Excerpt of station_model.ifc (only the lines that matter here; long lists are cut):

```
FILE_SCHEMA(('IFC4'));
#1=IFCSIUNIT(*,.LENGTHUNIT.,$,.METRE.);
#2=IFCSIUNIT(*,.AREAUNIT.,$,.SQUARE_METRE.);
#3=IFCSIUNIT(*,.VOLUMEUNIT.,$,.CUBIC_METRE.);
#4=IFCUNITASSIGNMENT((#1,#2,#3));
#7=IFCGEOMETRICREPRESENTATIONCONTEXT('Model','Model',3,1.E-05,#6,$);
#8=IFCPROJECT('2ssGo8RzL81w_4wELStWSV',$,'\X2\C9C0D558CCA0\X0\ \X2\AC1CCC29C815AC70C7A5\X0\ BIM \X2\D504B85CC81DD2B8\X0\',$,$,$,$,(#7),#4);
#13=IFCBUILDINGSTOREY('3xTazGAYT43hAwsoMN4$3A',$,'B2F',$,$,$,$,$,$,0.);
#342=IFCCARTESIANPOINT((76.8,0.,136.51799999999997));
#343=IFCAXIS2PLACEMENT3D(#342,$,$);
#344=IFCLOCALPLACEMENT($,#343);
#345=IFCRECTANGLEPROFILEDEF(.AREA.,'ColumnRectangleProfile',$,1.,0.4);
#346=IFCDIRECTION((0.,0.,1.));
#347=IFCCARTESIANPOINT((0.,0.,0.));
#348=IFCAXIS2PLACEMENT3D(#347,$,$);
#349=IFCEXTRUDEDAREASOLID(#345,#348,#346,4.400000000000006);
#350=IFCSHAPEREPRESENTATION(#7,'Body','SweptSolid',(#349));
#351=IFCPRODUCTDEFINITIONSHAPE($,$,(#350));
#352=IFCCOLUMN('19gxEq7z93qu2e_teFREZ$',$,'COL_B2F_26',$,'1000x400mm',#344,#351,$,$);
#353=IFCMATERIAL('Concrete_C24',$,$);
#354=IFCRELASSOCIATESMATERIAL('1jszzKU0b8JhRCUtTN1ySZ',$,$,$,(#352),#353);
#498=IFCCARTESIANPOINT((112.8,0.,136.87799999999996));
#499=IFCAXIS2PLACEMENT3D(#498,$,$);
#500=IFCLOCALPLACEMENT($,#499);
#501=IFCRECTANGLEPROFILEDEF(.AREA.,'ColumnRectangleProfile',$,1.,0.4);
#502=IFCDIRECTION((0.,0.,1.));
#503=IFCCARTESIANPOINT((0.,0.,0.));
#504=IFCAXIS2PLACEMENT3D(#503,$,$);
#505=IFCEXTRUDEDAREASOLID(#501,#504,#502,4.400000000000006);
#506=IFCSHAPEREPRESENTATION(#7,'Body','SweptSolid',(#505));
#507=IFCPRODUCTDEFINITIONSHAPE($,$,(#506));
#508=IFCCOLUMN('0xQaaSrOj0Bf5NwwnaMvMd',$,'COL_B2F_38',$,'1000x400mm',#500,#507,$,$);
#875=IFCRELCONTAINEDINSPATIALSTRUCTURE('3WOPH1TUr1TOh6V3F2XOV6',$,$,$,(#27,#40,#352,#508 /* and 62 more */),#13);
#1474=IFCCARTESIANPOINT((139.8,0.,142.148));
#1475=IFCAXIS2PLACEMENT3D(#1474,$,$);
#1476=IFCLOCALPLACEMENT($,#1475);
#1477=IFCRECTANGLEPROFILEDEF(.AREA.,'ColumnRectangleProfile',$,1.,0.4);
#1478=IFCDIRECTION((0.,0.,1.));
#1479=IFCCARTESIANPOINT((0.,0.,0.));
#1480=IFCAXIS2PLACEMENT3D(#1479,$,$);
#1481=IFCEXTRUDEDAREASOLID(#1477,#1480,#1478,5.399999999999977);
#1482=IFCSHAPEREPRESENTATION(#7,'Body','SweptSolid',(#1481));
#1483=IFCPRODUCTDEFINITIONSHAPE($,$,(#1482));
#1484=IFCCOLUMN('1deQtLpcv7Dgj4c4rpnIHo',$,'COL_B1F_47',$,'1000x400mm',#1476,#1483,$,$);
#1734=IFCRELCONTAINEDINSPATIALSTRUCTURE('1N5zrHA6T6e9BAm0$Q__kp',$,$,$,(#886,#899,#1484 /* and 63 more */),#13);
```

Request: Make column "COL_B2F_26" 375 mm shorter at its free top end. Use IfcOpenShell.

```python
import ifcopenshell
import ifcopenshell.util.unit

model = ifcopenshell.open("station_model.ifc")
unit_scale = ifcopenshell.util.unit.calculate_unit_scale(model)

member = model.by_guid("19gxEq7z93qu2e_teFREZ$")
change = -0.375 / unit_scale

# The extrusion runs towards the end named, so only its depth changes.
body = next(r for r in member.Representation.Representations if r.RepresentationIdentifier == "Body")
solid = body.Items[0]
old_length = solid.Depth
solid.Depth += change

print(f"length {old_length:g} -> {solid.Depth:g}")

model.write("station_model_rev.ifc")
```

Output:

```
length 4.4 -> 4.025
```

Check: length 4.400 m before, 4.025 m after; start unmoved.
